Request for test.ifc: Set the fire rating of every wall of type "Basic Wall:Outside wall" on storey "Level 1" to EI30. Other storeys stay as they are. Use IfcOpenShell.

First a look at what the model holds.

```python
import ifcopenshell
import ifcopenshell.util.element

model = ifcopenshell.open("test.ifc")
print(model.schema)
storey = next(s for s in model.by_type("IfcBuildingStorey") if s.Name == "Level 1")
walls = [e for e in ifcopenshell.util.element.get_decomposition(storey) if e.is_a("IfcWall")]
seen = {}
for e in walls:
    element_type = ifcopenshell.util.element.get_type(e)
    key = (element_type.Name if element_type != e and element_type else None, ifcopenshell.util.element.get_pset(e, "Pset_WallCommon", "FireRating"))
    seen[key] = seen.get(key, 0) + 1
for (name, value), count in sorted(seen.items(), key=str):
    print(count, "x", name, "|", value)
```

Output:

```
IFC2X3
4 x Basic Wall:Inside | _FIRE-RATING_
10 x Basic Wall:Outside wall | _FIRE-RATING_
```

```python
import ifcopenshell
import ifcopenshell.api.pset
import ifcopenshell.util.element

model = ifcopenshell.open("test.ifc")

storey = next(s for s in model.by_type("IfcBuildingStorey") if s.Name == "Level 1")
walls = [e for e in ifcopenshell.util.element.get_decomposition(storey) if e.is_a("IfcWall")]

count = 0
for e in walls:
    element_type = ifcopenshell.util.element.get_type(e)
    if element_type in (None, e) or element_type.Name != "Basic Wall:Outside wall":
        continue
    # add_pset returns the element's existing set when there is one.
    pset = ifcopenshell.api.pset.add_pset(model, product=e, name="Pset_WallCommon")
    ifcopenshell.api.pset.edit_pset(model, pset=pset, properties={"FireRating": "EI30"})
    count += 1

print(count, "walls updated")

model.write("test-out.ifc")
```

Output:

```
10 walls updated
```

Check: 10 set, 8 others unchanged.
